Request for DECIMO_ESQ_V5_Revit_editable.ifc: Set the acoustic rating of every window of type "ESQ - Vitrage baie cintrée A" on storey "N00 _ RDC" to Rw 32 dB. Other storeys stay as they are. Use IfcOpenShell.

First a look at what the model holds.

```python
import ifcopenshell
import ifcopenshell.util.element

model = ifcopenshell.open("DECIMO_ESQ_V5_Revit_editable.ifc")
print(model.schema)
storey = next(s for s in model.by_type("IfcBuildingStorey") if s.Name == "N00 _ RDC")
windows = [e for e in ifcopenshell.util.element.get_decomposition(storey) if e.is_a("IfcWindow")]
seen = {}
for e in windows:
    element_type = ifcopenshell.util.element.get_type(e)
    key = (element_type.Name if element_type != e and element_type else None, ifcopenshell.util.element.get_pset(e, "Pset_WindowCommon", "AcousticRating"))
    seen[key] = seen.get(key, 0) + 1
for (name, value), count in sorted(seen.items(), key=str):
    print(count, "x", name, "|", value)
```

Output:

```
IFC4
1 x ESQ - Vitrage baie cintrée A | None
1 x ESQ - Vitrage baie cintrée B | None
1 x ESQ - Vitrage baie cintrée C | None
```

```python
import ifcopenshell
import ifcopenshell.api.pset
import ifcopenshell.util.element

model = ifcopenshell.open("DECIMO_ESQ_V5_Revit_editable.ifc")

storey = next(s for s in model.by_type("IfcBuildingStorey") if s.Name == "N00 _ RDC")
windows = [e for e in ifcopenshell.util.element.get_decomposition(storey) if e.is_a("IfcWindow")]

count = 0
for e in windows:
    element_type = ifcopenshell.util.element.get_type(e)
    if element_type in (None, e) or element_type.Name != "ESQ - Vitrage baie cintrée A":
        continue
    # add_pset returns the element's existing set when there is one.
    pset = ifcopenshell.api.pset.add_pset(model, product=e, name="Pset_WindowCommon")
    ifcopenshell.api.pset.edit_pset(model, pset=pset, properties={"AcousticRating": "Rw 32 dB"})
    count += 1

print(count, "windows updated")

model.write("DECIMO_ESQ_V5_Revit_editable-out.ifc")
```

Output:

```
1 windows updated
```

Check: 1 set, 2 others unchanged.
